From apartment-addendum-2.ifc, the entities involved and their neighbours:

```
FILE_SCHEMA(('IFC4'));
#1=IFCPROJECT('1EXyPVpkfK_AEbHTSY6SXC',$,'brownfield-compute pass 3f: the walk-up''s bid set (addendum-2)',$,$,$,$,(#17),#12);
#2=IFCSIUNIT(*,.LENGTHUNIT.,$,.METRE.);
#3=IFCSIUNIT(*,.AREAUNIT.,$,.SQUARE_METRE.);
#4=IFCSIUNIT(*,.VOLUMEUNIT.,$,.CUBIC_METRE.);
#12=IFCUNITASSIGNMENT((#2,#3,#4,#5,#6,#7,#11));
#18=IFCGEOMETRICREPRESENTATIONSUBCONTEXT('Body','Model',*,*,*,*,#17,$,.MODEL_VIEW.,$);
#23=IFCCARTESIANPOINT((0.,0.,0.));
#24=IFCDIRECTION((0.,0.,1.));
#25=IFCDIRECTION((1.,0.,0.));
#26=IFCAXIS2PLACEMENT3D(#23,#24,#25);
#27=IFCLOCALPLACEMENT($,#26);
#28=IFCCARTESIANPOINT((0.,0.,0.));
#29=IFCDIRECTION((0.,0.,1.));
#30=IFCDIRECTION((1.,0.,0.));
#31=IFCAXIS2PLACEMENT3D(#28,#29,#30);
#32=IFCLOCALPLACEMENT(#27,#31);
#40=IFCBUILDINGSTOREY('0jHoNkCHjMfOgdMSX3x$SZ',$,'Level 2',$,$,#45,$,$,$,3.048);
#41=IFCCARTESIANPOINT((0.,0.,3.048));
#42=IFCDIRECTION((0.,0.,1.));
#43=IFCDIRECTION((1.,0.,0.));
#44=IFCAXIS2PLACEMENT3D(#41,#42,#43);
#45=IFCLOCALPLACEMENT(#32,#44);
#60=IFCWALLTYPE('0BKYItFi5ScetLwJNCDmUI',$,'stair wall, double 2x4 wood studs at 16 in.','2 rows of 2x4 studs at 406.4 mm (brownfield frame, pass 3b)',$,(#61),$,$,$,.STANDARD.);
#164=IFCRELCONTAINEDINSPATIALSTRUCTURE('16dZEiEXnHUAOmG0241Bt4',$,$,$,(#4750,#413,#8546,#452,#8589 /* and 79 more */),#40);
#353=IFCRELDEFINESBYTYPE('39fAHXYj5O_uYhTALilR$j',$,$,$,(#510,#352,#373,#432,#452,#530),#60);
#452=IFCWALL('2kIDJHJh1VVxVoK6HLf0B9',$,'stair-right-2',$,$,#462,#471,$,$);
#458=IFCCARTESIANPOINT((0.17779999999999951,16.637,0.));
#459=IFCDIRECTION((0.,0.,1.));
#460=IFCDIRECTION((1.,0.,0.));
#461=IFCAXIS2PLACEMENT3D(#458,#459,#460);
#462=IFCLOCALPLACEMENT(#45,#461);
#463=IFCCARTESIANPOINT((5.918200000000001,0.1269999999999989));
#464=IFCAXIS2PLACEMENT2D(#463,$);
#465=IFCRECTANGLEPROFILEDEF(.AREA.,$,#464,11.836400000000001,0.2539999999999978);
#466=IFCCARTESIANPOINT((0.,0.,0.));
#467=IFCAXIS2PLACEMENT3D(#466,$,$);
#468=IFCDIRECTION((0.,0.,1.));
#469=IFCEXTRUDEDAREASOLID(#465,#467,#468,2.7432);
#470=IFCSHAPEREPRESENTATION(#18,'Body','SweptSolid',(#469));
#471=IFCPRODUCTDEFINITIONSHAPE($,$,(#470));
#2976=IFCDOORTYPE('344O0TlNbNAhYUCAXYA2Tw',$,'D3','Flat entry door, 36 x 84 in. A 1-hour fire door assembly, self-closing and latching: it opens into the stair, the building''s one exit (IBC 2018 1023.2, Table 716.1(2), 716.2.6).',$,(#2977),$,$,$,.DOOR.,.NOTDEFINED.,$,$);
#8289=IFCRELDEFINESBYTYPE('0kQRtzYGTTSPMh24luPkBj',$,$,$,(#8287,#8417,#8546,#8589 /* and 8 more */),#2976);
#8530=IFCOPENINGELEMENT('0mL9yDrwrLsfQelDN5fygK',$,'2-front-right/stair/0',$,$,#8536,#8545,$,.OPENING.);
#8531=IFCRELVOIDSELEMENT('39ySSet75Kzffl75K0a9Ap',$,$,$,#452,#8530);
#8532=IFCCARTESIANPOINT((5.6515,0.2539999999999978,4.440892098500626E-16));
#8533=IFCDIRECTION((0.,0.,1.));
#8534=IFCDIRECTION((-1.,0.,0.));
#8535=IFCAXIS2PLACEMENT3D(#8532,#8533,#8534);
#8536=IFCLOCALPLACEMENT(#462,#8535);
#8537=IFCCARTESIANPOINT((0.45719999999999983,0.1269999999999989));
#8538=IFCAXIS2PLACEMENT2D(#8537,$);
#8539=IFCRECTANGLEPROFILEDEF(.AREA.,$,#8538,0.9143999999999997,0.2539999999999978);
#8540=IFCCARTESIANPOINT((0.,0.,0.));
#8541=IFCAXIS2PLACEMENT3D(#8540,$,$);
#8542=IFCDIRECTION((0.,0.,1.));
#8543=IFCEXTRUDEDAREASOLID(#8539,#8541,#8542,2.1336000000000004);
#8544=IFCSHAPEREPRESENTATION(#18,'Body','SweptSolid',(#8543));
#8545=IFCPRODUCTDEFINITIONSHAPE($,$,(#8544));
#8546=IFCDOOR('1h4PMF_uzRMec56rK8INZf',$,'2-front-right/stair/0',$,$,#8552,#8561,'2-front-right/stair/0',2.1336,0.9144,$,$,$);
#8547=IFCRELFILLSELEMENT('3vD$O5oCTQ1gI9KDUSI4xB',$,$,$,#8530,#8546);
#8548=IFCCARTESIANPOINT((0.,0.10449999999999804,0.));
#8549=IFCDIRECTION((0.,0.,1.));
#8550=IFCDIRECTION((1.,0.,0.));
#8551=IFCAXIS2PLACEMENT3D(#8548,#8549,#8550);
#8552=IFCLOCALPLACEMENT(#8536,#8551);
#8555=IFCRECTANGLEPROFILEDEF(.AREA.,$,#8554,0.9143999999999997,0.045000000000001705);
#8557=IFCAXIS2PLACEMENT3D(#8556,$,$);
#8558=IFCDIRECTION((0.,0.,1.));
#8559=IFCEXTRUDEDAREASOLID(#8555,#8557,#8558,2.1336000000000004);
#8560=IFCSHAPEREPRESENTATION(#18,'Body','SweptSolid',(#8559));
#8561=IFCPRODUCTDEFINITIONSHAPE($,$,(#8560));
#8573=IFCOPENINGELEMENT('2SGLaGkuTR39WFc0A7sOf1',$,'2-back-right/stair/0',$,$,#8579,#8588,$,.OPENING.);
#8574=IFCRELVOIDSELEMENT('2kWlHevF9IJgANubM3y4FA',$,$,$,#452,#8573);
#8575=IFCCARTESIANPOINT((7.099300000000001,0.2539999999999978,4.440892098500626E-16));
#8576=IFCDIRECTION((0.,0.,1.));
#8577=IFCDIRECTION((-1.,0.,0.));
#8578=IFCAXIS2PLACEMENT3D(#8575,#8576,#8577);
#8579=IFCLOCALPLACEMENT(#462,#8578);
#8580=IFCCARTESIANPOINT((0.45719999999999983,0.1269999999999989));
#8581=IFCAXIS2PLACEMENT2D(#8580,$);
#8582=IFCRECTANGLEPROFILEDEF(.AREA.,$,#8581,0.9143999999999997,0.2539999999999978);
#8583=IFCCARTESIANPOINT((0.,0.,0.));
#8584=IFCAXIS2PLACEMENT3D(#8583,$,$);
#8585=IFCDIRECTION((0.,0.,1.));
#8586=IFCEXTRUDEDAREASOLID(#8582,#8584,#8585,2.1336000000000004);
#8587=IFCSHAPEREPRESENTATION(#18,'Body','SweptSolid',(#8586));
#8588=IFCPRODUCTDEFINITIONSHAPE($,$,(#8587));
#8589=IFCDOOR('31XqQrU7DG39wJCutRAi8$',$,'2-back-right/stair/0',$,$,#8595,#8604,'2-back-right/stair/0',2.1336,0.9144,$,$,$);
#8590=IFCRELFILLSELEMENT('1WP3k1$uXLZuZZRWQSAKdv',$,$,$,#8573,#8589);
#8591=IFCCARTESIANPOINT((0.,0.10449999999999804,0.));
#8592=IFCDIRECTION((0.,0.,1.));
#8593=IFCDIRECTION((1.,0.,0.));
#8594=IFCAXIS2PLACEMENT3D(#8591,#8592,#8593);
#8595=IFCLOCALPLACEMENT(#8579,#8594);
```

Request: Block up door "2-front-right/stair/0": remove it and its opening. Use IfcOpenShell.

```python
import ifcopenshell
import ifcopenshell.api.feature
import ifcopenshell.api.root
import ifcopenshell.geom
import ifcopenshell.util.shape

model = ifcopenshell.open("apartment-addendum-2.ifc")
settings = ifcopenshell.geom.settings()


def volume(element):
    """Net volume in cubic metres, openings subtracted."""
    shape = ifcopenshell.geom.create_shape(settings, element)
    return ifcopenshell.util.shape.get_volume(shape.geometry)


door = model.by_id(8546)
opening = door.FillsVoids[0].RelatingOpeningElement
wall = opening.VoidsElements[0].RelatingBuildingElement
before = volume(wall)

ifcopenshell.api.root.remove_product(model, product=door)
ifcopenshell.api.feature.remove_feature(model, feature=opening)

after = volume(wall)

print(f"wall volume {before:.3f} -> {after:.3f} m3")

model.write("apartment-addendum-2_v2.ifc")
```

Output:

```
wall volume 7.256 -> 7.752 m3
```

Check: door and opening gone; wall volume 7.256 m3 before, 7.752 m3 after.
